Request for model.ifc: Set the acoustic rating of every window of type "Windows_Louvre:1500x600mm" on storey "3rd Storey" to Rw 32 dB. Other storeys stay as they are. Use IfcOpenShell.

First a look at what the model holds.

```python
import ifcopenshell
import ifcopenshell.util.element

model = ifcopenshell.open("model.ifc")
print(model.schema)
storey = next(s for s in model.by_type("IfcBuildingStorey") if s.Name == "3rd Storey")
windows = [e for e in ifcopenshell.util.element.get_decomposition(storey) if e.is_a("IfcWindow")]
seen = {}
for e in windows:
    element_type = ifcopenshell.util.element.get_type(e)
    key = (element_type.Name if element_type != e and element_type else None, ifcopenshell.util.element.get_pset(e, "Pset_WindowCommon", "AcousticRating"))
    seen[key] = seen.get(key, 0) + 1
for (name, value), count in sorted(seen.items(), key=str):
    print(count, "x", name, "|", value)
```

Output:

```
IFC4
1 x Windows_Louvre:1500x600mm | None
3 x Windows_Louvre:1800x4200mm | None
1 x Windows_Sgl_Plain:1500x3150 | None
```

```python
import ifcopenshell
import ifcopenshell.api.pset
import ifcopenshell.util.element

model = ifcopenshell.open("model.ifc")

storey = next(s for s in model.by_type("IfcBuildingStorey") if s.Name == "3rd Storey")
windows = [e for e in ifcopenshell.util.element.get_decomposition(storey) if e.is_a("IfcWindow")]

count = 0
for e in windows:
    element_type = ifcopenshell.util.element.get_type(e)
    if element_type in (None, e) or element_type.Name != "Windows_Louvre:1500x600mm":
        continue
    # add_pset returns the element's existing set when there is one.
    pset = ifcopenshell.api.pset.add_pset(model, product=e, name="Pset_WindowCommon")
    ifcopenshell.api.pset.edit_pset(model, pset=pset, properties={"AcousticRating": "Rw 32 dB"})
    count += 1

print(count, "windows updated")

model.write("model_v2.ifc")
```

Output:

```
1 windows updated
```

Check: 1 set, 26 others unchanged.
